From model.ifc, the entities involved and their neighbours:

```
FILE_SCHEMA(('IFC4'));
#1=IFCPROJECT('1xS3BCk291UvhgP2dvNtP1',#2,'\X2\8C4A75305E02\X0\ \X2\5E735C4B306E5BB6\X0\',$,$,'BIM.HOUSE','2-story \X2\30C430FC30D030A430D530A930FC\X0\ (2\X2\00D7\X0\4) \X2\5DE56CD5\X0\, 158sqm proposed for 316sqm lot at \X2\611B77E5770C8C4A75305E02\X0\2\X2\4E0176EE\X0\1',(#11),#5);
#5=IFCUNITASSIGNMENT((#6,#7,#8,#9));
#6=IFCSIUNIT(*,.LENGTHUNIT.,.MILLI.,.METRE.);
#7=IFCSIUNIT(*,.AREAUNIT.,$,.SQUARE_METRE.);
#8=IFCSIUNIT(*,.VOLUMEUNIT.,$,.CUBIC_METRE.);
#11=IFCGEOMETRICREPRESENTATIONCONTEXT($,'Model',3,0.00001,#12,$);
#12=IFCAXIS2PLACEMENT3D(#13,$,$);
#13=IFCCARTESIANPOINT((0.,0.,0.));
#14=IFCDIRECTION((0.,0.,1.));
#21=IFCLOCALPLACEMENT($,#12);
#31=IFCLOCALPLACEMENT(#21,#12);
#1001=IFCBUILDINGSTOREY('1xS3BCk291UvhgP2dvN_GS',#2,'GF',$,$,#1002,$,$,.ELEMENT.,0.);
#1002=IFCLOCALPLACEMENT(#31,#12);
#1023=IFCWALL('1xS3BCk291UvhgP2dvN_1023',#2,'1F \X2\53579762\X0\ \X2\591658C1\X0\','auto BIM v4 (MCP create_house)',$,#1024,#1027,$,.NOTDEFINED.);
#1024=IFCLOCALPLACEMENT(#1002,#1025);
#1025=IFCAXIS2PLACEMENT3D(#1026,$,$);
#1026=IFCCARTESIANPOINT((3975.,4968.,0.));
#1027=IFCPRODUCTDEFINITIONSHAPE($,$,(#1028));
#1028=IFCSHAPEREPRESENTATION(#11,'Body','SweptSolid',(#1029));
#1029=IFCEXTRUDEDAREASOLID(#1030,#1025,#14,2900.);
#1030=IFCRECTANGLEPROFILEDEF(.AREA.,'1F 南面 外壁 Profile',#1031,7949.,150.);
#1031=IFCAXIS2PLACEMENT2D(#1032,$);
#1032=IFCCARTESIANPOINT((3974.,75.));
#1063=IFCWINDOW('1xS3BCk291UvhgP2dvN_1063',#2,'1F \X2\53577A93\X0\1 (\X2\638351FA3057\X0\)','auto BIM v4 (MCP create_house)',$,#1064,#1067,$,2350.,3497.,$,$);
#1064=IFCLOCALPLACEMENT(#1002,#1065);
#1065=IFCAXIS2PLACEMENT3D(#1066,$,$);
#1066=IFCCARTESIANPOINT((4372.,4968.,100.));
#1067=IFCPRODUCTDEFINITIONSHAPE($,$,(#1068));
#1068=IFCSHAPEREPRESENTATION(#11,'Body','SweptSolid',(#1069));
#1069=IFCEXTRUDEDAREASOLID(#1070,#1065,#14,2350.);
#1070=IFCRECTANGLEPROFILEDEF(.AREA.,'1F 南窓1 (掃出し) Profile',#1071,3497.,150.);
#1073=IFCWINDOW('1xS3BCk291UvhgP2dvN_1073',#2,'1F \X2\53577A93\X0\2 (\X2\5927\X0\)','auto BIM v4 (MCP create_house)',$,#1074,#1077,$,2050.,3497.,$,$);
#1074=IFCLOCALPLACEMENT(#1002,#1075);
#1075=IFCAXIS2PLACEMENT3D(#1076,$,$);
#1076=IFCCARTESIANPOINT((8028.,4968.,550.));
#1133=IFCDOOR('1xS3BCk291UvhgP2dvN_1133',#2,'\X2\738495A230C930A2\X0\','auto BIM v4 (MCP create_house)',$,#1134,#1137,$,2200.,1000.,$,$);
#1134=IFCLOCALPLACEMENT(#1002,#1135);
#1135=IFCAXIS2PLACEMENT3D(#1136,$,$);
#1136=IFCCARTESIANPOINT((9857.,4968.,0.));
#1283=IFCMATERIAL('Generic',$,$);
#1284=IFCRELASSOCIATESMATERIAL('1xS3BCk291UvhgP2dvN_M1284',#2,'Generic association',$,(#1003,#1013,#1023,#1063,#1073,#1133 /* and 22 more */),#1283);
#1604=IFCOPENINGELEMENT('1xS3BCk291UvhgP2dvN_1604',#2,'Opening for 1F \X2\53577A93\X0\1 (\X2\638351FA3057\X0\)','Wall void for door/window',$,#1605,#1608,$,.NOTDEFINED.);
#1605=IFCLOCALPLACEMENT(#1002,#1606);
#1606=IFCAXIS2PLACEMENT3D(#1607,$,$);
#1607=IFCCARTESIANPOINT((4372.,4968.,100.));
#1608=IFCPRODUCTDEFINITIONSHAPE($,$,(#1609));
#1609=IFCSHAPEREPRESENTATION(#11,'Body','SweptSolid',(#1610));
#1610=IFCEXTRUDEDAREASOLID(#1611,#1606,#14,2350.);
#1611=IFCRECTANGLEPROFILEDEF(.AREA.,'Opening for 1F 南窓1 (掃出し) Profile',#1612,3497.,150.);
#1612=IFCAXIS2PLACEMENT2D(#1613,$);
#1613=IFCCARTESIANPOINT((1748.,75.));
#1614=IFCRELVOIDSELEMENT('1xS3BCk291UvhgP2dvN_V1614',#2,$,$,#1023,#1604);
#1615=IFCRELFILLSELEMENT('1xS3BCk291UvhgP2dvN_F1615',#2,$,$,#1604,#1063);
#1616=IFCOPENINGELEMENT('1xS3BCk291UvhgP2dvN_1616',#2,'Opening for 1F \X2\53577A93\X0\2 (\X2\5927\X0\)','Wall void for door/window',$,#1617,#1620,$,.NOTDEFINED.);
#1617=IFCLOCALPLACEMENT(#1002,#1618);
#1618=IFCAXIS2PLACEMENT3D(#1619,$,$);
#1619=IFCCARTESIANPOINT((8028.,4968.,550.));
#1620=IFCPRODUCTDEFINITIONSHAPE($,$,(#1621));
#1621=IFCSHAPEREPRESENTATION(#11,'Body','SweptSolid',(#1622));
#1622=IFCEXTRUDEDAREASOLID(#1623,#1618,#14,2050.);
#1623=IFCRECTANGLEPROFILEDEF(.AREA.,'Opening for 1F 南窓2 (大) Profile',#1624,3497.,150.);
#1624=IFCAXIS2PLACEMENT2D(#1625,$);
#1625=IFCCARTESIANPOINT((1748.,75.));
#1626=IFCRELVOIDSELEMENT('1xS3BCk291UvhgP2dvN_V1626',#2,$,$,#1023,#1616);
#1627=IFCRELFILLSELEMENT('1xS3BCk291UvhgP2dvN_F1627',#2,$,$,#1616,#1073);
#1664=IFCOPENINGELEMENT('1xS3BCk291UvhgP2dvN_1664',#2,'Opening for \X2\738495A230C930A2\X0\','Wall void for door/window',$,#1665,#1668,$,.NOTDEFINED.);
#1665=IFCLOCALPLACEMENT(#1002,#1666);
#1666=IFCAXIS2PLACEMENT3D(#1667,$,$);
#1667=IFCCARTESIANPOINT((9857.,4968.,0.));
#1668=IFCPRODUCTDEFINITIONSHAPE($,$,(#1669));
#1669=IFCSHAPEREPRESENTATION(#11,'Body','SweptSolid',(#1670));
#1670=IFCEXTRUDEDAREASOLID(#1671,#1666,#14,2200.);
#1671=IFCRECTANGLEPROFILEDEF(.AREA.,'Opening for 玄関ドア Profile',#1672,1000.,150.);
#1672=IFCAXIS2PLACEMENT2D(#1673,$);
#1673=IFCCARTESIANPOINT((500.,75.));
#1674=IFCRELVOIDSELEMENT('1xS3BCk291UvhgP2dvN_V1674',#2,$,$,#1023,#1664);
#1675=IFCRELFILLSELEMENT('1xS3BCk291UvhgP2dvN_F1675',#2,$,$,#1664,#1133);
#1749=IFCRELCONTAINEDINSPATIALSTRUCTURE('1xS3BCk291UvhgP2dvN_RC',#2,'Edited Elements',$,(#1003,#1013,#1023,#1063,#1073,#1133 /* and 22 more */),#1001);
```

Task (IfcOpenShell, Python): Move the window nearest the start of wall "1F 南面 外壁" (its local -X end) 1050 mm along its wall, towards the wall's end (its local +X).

```python
import ifcopenshell
import ifcopenshell.api.geometry
import ifcopenshell.util.placement
import ifcopenshell.util.unit

model = ifcopenshell.open("model.ifc")
unit_scale = ifcopenshell.util.unit.calculate_unit_scale(model)

window = model.by_id(1063)
opening = window.FillsVoids[0].RelatingOpeningElement
wall = opening.VoidsElements[0].RelatingBuildingElement

wall_matrix = ifcopenshell.util.placement.get_local_placement(wall.ObjectPlacement)
shift = wall_matrix[:3, 0] * 1.05 / unit_scale
before = ifcopenshell.util.placement.get_local_placement(window.ObjectPlacement)[:3, 3].copy()

# The window is not placed relative to its opening, so move both.
for product in (opening, window):
    matrix = ifcopenshell.util.placement.get_local_placement(product.ObjectPlacement)
    matrix[:3, 3] += shift
    ifcopenshell.api.geometry.edit_object_placement(model, product=product, matrix=matrix, is_si=False)

after = ifcopenshell.util.placement.get_local_placement(window.ObjectPlacement)[:3, 3]
print("window moved by", (after - before).round(3) + 0.0)

model.write("model_rev.ifc")
```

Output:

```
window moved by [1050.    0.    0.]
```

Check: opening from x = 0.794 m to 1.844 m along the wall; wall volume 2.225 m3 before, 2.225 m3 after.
